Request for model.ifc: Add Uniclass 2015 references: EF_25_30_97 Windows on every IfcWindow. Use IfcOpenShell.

First a look at what the model holds.

```python
import ifcopenshell

model = ifcopenshell.open("model.ifc")
print(model.schema)
print("classifications:", [c.Name for c in model.by_type("IfcClassification")])
for ifc_class in ("IfcDoor", "IfcRoof", "IfcStair", "IfcWall", "IfcWindow"):
    print(ifc_class, len(model.by_type(ifc_class)))
```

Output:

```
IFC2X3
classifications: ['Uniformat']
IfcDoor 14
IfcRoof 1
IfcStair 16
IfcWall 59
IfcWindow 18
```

```python
import ifcopenshell
import ifcopenshell.api.classification

model = ifcopenshell.open("model.ifc")

# IFC2X3 requires Source and Edition and has no link from the project to the system.
system = model.create_entity("IfcClassification", Source="NBS", Edition="2015", Name="Uniclass 2015")

codes = {
    "IfcWindow": ("EF_25_30_97", "Windows"),
}
for ifc_class, (code, name) in codes.items():
    products = model.by_type(ifc_class)
    ifcopenshell.api.classification.add_reference(
        model, products=products, classification=system, identification=code, name=name
    )
    print(code, len(products))

model.write("model_updated.ifc")
```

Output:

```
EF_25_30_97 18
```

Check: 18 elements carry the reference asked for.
